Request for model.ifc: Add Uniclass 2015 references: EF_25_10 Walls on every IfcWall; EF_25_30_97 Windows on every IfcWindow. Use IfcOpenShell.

First a look at what the model holds.

```python
import ifcopenshell

model = ifcopenshell.open("model.ifc")
print(model.schema)
print("classifications:", [c.Name for c in model.by_type("IfcClassification")])
for ifc_class in ("IfcDoor", "IfcRoof", "IfcStair", "IfcWall", "IfcWindow"):
    print(ifc_class, len(model.by_type(ifc_class)))
```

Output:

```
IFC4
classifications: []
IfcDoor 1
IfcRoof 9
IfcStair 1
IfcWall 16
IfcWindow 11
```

```python
import ifcopenshell
import ifcopenshell.api.classification

model = ifcopenshell.open("model.ifc")

system = ifcopenshell.api.classification.add_classification(model, classification="Uniclass 2015")

codes = {
    "IfcWall": ("EF_25_10", "Walls"),
    "IfcWindow": ("EF_25_30_97", "Windows"),
}
for ifc_class, (code, name) in codes.items():
    products = model.by_type(ifc_class)
    ifcopenshell.api.classification.add_reference(
        model, products=products, classification=system, identification=code, name=name
    )
    print(code, len(products))

model.write("model_rev.ifc")
```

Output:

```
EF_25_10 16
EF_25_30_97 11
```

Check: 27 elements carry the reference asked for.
